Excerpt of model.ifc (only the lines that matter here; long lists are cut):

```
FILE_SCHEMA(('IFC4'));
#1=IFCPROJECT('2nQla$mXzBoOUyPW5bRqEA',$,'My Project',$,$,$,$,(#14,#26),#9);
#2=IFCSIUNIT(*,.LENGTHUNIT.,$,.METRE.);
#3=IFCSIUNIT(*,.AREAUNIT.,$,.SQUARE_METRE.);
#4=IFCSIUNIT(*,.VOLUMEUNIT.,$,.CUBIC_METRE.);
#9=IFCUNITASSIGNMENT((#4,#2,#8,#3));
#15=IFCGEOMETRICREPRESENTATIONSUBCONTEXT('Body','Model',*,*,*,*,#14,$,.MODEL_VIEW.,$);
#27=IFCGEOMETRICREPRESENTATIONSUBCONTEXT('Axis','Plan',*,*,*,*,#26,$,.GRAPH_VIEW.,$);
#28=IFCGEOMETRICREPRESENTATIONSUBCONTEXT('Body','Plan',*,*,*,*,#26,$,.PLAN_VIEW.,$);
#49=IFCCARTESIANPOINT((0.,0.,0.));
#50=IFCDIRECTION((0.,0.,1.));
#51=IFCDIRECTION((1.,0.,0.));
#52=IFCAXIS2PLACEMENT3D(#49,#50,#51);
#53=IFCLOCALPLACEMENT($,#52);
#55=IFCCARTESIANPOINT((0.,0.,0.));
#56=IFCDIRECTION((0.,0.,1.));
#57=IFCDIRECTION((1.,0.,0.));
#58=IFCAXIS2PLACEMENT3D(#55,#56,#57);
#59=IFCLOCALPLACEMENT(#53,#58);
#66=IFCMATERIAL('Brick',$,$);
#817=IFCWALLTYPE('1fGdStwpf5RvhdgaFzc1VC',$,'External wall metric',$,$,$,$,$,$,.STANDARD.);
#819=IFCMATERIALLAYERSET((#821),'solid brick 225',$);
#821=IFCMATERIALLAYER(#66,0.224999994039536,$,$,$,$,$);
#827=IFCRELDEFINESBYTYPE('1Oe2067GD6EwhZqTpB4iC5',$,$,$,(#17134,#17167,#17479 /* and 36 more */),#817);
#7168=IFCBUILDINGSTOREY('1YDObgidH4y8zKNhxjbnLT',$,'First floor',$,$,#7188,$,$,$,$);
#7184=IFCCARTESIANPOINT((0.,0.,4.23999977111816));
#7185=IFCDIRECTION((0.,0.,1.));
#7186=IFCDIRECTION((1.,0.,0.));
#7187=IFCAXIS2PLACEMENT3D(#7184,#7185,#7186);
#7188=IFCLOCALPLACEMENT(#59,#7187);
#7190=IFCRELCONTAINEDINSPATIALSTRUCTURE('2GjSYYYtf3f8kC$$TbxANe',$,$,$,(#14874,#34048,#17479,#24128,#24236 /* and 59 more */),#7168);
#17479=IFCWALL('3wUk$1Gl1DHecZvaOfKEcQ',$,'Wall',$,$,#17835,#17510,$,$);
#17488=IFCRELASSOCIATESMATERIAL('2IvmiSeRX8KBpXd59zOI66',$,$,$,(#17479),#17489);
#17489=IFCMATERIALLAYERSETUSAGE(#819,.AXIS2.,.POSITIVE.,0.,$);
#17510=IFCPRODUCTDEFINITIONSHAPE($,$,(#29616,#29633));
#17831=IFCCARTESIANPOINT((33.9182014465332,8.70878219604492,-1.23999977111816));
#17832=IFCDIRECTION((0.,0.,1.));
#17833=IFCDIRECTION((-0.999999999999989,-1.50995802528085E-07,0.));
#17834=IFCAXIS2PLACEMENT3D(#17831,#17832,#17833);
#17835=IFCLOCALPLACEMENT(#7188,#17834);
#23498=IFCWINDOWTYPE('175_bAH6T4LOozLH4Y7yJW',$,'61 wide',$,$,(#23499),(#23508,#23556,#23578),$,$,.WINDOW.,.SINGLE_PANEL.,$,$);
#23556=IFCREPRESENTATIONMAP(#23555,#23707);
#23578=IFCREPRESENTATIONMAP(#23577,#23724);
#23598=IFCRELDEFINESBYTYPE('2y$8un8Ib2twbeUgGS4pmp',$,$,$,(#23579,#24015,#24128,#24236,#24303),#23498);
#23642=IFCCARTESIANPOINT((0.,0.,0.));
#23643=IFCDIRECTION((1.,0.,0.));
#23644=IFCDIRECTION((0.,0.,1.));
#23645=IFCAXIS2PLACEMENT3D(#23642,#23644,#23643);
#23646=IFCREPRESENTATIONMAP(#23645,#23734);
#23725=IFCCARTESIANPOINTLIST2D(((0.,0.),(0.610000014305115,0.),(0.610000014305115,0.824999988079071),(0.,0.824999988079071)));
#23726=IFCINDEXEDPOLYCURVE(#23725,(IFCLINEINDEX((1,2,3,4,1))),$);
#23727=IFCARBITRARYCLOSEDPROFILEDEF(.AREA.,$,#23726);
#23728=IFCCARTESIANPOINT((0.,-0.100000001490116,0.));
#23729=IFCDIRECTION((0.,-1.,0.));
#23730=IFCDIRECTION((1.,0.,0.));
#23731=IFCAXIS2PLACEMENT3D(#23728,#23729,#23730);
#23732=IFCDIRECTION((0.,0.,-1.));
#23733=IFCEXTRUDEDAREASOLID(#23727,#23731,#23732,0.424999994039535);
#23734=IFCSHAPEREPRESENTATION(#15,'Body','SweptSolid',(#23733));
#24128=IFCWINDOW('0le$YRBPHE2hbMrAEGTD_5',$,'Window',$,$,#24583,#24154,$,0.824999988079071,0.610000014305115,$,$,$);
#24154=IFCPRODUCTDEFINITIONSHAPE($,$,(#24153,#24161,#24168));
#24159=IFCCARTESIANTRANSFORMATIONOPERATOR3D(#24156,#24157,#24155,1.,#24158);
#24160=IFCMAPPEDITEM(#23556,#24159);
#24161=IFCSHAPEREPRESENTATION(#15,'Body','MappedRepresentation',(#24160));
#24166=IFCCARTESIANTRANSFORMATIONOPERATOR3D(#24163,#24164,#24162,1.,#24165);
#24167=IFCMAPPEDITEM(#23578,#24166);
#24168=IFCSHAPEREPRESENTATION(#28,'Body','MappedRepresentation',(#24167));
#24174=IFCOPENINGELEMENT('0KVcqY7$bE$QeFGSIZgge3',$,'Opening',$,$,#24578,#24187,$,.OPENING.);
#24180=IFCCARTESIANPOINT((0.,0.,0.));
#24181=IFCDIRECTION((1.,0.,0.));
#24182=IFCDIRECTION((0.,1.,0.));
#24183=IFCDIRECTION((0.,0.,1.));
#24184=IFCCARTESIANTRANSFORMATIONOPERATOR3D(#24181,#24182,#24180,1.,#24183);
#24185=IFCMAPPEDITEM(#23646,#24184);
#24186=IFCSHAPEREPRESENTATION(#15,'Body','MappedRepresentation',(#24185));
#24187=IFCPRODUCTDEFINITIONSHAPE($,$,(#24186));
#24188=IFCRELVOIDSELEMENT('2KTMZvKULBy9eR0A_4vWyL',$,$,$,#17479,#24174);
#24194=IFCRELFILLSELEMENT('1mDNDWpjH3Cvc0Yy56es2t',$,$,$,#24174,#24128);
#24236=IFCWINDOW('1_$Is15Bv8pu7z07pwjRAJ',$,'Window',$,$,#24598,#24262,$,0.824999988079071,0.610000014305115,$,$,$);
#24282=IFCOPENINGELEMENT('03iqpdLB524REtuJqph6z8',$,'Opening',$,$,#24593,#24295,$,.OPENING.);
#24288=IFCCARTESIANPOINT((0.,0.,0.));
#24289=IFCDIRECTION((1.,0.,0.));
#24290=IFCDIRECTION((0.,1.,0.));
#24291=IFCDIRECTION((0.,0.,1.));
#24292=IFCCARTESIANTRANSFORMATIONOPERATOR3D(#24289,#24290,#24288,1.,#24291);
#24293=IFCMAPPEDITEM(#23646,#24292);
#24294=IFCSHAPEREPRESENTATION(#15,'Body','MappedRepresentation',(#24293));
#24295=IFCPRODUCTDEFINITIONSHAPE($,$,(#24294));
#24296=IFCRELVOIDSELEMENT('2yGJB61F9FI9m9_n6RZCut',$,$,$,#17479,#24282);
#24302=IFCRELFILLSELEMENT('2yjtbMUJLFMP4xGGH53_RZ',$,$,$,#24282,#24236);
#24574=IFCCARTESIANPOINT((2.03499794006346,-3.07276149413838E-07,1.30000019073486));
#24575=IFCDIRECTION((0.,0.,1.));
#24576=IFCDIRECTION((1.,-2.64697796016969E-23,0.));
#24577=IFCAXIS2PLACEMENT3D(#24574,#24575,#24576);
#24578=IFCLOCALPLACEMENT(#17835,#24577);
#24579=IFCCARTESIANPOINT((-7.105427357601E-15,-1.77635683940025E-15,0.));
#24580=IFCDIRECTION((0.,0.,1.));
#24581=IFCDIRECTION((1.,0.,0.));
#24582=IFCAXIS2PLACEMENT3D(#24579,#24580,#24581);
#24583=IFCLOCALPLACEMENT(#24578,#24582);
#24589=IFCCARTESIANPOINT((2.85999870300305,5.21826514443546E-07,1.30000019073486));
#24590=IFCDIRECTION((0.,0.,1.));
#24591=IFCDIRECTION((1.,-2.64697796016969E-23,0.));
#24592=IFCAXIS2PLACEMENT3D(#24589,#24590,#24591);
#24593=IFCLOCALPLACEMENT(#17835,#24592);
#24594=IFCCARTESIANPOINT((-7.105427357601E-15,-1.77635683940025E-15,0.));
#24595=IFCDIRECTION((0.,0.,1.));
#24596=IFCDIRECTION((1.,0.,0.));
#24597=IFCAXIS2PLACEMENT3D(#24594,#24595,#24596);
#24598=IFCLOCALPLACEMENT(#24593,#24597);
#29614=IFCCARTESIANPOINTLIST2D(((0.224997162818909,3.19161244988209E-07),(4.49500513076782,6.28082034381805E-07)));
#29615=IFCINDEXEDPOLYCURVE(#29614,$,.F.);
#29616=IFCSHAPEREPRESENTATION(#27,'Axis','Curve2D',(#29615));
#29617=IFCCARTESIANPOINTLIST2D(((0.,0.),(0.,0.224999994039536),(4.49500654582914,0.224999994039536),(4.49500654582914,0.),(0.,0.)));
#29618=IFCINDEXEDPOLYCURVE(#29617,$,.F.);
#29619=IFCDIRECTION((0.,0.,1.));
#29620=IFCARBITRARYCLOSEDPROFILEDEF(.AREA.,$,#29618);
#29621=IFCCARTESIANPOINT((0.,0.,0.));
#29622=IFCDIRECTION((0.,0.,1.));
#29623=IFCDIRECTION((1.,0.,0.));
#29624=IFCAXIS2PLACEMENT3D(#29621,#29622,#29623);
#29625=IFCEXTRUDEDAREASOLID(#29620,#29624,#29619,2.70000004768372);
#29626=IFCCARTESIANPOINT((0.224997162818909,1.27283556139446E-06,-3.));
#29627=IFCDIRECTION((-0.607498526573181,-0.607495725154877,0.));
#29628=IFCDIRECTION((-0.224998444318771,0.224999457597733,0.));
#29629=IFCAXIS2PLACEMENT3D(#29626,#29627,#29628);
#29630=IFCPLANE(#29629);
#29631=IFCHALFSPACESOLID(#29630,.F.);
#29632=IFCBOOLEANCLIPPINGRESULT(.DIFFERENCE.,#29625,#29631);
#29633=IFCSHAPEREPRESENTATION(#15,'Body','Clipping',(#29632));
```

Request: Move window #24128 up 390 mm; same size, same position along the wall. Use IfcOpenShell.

```python
import numpy as np
import ifcopenshell
import ifcopenshell.api.geometry
import ifcopenshell.util.placement
import ifcopenshell.util.unit

model = ifcopenshell.open("model.ifc")
unit_scale = ifcopenshell.util.unit.calculate_unit_scale(model)

window = model.by_guid("0le$YRBPHE2hbMrAEGTD_5")
opening = window.FillsVoids[0].RelatingOpeningElement
dz = 0.39

shift = np.array([0.0, 0.0, dz])
# The window is placed relative to its opening, so it follows when the opening moves.
matrix = ifcopenshell.util.placement.get_local_placement(opening.ObjectPlacement)
matrix[:3, 3] += shift
ifcopenshell.api.geometry.edit_object_placement(
    model, product=opening, matrix=matrix, is_si=False, should_transform_children=True
)

print(f"moved by {dz * unit_scale:+.3f} m")

model.write("model_edited.ifc")
```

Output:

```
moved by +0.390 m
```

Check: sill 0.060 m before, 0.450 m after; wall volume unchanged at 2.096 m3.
